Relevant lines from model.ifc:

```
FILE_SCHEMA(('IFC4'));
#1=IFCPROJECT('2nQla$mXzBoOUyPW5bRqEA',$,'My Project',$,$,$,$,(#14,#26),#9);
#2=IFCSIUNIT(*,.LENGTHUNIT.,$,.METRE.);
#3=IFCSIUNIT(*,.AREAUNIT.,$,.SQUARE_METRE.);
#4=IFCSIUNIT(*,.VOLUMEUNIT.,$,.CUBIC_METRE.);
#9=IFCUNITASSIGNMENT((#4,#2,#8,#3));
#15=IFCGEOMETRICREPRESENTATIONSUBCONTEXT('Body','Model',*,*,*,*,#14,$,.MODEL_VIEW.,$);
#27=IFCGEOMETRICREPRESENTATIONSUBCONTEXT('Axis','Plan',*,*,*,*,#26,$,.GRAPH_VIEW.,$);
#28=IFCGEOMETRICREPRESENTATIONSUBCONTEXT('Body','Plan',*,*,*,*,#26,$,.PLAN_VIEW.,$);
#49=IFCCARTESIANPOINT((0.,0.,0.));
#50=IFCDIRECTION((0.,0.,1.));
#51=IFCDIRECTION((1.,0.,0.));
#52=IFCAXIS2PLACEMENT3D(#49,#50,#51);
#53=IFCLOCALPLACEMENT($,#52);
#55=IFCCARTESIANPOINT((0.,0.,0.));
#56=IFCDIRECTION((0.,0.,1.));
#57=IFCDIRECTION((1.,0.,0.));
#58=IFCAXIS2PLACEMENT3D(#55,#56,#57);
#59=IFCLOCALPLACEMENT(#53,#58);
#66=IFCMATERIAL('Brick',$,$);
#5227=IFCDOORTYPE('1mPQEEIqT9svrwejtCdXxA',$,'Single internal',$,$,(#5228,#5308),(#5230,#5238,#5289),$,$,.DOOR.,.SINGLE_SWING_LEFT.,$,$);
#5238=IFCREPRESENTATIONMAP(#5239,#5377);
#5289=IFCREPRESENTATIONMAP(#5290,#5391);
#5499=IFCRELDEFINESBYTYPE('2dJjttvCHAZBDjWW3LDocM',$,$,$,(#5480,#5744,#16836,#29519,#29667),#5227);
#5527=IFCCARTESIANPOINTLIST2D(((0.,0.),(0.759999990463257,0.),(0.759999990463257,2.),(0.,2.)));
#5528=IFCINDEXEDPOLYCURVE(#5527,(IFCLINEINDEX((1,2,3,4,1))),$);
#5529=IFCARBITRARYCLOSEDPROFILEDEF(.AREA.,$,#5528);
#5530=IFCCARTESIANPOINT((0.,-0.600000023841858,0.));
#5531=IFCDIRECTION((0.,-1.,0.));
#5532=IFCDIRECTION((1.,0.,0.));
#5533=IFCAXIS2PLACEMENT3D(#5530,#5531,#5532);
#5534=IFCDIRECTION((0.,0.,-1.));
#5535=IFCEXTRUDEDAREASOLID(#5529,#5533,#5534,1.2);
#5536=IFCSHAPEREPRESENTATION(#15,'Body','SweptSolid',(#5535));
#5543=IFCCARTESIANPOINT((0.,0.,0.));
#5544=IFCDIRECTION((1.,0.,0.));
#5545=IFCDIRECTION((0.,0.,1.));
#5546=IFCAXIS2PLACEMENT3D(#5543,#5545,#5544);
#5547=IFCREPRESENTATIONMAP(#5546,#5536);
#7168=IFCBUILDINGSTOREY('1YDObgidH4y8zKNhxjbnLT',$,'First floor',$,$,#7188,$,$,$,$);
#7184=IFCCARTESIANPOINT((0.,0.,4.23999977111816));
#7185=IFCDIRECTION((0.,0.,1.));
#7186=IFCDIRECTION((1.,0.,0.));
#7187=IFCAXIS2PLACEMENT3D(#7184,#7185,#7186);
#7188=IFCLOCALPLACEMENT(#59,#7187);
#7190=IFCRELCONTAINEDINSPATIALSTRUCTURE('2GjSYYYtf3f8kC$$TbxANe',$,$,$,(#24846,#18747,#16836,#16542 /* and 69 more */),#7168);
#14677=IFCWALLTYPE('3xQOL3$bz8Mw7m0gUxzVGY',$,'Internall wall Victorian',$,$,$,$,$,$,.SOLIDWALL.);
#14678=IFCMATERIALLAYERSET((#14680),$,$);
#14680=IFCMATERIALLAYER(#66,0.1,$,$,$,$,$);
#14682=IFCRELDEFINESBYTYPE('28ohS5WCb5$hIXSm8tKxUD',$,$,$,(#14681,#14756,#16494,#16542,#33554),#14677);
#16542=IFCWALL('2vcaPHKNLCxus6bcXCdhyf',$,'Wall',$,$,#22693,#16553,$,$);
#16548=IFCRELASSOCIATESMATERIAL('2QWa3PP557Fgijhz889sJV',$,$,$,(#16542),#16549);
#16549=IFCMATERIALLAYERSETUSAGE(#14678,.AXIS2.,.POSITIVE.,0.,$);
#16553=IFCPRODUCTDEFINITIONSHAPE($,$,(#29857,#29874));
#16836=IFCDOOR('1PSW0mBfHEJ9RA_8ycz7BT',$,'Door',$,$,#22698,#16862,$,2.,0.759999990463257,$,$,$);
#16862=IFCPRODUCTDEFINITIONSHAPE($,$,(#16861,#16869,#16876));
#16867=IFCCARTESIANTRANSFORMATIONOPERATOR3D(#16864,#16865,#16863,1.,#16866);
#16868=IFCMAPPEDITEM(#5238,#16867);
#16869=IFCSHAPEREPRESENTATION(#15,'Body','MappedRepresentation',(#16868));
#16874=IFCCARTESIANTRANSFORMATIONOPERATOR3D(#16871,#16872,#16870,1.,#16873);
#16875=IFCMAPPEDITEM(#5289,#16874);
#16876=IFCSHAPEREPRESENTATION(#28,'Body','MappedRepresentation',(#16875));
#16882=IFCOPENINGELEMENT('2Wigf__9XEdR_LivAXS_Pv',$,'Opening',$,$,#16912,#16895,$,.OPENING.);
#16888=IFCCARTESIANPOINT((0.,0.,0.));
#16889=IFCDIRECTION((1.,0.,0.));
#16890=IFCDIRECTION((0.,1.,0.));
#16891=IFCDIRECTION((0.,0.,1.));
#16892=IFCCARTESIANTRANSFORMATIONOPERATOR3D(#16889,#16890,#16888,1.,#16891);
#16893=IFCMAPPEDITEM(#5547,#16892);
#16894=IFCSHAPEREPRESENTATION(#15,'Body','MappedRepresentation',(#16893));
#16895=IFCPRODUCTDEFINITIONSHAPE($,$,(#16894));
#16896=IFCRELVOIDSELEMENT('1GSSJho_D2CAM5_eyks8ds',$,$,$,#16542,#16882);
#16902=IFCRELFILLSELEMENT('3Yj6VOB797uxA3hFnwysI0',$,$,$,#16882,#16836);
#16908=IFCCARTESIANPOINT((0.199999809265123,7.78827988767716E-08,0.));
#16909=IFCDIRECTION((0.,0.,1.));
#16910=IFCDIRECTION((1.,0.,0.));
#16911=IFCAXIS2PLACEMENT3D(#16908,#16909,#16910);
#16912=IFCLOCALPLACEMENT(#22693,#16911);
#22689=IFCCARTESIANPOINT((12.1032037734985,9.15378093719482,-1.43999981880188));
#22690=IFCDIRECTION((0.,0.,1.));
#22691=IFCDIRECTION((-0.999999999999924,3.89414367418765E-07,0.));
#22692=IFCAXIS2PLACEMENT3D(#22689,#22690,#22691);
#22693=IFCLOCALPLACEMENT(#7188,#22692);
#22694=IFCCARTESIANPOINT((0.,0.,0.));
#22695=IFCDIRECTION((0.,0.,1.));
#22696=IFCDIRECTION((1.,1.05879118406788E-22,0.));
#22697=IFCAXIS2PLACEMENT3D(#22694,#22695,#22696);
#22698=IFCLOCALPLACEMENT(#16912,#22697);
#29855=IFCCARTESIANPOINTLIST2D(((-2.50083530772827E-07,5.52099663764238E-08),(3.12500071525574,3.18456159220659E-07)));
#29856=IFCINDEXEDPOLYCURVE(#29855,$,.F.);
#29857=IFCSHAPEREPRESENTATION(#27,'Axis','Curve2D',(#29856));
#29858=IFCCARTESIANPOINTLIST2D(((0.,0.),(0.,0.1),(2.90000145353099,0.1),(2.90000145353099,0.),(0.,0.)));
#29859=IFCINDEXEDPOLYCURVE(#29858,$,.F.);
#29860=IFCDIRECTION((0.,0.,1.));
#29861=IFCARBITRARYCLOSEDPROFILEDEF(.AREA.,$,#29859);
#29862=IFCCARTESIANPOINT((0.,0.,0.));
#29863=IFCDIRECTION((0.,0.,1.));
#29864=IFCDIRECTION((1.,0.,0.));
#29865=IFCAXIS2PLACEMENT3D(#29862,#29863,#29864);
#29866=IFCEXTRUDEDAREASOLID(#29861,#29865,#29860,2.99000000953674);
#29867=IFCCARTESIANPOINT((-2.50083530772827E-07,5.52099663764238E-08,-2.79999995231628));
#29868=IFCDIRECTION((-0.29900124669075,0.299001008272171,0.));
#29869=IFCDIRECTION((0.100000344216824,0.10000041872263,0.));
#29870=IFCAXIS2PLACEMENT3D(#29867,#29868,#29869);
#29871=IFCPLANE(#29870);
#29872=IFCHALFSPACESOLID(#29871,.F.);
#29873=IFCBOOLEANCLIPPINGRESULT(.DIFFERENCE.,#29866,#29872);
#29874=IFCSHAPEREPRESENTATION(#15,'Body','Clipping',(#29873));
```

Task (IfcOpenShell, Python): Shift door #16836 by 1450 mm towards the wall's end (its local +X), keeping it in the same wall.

```python
import ifcopenshell
import ifcopenshell.api.geometry
import ifcopenshell.util.placement
import ifcopenshell.util.unit

model = ifcopenshell.open("model.ifc")
unit_scale = ifcopenshell.util.unit.calculate_unit_scale(model)

door = model.by_guid("1PSW0mBfHEJ9RA_8ycz7BT")
opening = door.FillsVoids[0].RelatingOpeningElement
wall = opening.VoidsElements[0].RelatingBuildingElement

wall_matrix = ifcopenshell.util.placement.get_local_placement(wall.ObjectPlacement)
shift = wall_matrix[:3, 0] * 1.45 / unit_scale
before = ifcopenshell.util.placement.get_local_placement(door.ObjectPlacement)[:3, 3].copy()

# The door is placed relative to its opening, so it follows when the opening moves.
matrix = ifcopenshell.util.placement.get_local_placement(opening.ObjectPlacement)
matrix[:3, 3] += shift
ifcopenshell.api.geometry.edit_object_placement(
    model, product=opening, matrix=matrix, is_si=False, should_transform_children=True
)

after = ifcopenshell.util.placement.get_local_placement(door.ObjectPlacement)[:3, 3]
print("door moved by", (after - before).round(3) + 0.0)

model.write("model_rev.ifc")
```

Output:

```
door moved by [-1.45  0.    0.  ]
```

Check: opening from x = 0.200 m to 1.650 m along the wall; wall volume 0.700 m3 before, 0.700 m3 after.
